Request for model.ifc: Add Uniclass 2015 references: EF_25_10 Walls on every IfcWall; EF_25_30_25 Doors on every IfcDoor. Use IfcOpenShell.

First a look at what the model holds.

```python
import ifcopenshell

model = ifcopenshell.open("model.ifc")
print(model.schema)
print("classifications:", [c.Name for c in model.by_type("IfcClassification")])
for ifc_class in ("IfcDoor", "IfcRoof", "IfcStair", "IfcWall", "IfcWindow"):
    print(ifc_class, len(model.by_type(ifc_class)))
```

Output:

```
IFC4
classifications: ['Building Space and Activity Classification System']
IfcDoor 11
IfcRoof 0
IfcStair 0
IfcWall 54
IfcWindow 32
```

```python
import ifcopenshell
import ifcopenshell.api.classification

model = ifcopenshell.open("model.ifc")

system = ifcopenshell.api.classification.add_classification(model, classification="Uniclass 2015")

codes = {
    "IfcWall": ("EF_25_10", "Walls"),
    "IfcDoor": ("EF_25_30_25", "Doors"),
}
for ifc_class, (code, name) in codes.items():
    products = model.by_type(ifc_class)
    ifcopenshell.api.classification.add_reference(
        model, products=products, classification=system, identification=code, name=name
    )
    print(code, len(products))

model.write("model_v2.ifc")
```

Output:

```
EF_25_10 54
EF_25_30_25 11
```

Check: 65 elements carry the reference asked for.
